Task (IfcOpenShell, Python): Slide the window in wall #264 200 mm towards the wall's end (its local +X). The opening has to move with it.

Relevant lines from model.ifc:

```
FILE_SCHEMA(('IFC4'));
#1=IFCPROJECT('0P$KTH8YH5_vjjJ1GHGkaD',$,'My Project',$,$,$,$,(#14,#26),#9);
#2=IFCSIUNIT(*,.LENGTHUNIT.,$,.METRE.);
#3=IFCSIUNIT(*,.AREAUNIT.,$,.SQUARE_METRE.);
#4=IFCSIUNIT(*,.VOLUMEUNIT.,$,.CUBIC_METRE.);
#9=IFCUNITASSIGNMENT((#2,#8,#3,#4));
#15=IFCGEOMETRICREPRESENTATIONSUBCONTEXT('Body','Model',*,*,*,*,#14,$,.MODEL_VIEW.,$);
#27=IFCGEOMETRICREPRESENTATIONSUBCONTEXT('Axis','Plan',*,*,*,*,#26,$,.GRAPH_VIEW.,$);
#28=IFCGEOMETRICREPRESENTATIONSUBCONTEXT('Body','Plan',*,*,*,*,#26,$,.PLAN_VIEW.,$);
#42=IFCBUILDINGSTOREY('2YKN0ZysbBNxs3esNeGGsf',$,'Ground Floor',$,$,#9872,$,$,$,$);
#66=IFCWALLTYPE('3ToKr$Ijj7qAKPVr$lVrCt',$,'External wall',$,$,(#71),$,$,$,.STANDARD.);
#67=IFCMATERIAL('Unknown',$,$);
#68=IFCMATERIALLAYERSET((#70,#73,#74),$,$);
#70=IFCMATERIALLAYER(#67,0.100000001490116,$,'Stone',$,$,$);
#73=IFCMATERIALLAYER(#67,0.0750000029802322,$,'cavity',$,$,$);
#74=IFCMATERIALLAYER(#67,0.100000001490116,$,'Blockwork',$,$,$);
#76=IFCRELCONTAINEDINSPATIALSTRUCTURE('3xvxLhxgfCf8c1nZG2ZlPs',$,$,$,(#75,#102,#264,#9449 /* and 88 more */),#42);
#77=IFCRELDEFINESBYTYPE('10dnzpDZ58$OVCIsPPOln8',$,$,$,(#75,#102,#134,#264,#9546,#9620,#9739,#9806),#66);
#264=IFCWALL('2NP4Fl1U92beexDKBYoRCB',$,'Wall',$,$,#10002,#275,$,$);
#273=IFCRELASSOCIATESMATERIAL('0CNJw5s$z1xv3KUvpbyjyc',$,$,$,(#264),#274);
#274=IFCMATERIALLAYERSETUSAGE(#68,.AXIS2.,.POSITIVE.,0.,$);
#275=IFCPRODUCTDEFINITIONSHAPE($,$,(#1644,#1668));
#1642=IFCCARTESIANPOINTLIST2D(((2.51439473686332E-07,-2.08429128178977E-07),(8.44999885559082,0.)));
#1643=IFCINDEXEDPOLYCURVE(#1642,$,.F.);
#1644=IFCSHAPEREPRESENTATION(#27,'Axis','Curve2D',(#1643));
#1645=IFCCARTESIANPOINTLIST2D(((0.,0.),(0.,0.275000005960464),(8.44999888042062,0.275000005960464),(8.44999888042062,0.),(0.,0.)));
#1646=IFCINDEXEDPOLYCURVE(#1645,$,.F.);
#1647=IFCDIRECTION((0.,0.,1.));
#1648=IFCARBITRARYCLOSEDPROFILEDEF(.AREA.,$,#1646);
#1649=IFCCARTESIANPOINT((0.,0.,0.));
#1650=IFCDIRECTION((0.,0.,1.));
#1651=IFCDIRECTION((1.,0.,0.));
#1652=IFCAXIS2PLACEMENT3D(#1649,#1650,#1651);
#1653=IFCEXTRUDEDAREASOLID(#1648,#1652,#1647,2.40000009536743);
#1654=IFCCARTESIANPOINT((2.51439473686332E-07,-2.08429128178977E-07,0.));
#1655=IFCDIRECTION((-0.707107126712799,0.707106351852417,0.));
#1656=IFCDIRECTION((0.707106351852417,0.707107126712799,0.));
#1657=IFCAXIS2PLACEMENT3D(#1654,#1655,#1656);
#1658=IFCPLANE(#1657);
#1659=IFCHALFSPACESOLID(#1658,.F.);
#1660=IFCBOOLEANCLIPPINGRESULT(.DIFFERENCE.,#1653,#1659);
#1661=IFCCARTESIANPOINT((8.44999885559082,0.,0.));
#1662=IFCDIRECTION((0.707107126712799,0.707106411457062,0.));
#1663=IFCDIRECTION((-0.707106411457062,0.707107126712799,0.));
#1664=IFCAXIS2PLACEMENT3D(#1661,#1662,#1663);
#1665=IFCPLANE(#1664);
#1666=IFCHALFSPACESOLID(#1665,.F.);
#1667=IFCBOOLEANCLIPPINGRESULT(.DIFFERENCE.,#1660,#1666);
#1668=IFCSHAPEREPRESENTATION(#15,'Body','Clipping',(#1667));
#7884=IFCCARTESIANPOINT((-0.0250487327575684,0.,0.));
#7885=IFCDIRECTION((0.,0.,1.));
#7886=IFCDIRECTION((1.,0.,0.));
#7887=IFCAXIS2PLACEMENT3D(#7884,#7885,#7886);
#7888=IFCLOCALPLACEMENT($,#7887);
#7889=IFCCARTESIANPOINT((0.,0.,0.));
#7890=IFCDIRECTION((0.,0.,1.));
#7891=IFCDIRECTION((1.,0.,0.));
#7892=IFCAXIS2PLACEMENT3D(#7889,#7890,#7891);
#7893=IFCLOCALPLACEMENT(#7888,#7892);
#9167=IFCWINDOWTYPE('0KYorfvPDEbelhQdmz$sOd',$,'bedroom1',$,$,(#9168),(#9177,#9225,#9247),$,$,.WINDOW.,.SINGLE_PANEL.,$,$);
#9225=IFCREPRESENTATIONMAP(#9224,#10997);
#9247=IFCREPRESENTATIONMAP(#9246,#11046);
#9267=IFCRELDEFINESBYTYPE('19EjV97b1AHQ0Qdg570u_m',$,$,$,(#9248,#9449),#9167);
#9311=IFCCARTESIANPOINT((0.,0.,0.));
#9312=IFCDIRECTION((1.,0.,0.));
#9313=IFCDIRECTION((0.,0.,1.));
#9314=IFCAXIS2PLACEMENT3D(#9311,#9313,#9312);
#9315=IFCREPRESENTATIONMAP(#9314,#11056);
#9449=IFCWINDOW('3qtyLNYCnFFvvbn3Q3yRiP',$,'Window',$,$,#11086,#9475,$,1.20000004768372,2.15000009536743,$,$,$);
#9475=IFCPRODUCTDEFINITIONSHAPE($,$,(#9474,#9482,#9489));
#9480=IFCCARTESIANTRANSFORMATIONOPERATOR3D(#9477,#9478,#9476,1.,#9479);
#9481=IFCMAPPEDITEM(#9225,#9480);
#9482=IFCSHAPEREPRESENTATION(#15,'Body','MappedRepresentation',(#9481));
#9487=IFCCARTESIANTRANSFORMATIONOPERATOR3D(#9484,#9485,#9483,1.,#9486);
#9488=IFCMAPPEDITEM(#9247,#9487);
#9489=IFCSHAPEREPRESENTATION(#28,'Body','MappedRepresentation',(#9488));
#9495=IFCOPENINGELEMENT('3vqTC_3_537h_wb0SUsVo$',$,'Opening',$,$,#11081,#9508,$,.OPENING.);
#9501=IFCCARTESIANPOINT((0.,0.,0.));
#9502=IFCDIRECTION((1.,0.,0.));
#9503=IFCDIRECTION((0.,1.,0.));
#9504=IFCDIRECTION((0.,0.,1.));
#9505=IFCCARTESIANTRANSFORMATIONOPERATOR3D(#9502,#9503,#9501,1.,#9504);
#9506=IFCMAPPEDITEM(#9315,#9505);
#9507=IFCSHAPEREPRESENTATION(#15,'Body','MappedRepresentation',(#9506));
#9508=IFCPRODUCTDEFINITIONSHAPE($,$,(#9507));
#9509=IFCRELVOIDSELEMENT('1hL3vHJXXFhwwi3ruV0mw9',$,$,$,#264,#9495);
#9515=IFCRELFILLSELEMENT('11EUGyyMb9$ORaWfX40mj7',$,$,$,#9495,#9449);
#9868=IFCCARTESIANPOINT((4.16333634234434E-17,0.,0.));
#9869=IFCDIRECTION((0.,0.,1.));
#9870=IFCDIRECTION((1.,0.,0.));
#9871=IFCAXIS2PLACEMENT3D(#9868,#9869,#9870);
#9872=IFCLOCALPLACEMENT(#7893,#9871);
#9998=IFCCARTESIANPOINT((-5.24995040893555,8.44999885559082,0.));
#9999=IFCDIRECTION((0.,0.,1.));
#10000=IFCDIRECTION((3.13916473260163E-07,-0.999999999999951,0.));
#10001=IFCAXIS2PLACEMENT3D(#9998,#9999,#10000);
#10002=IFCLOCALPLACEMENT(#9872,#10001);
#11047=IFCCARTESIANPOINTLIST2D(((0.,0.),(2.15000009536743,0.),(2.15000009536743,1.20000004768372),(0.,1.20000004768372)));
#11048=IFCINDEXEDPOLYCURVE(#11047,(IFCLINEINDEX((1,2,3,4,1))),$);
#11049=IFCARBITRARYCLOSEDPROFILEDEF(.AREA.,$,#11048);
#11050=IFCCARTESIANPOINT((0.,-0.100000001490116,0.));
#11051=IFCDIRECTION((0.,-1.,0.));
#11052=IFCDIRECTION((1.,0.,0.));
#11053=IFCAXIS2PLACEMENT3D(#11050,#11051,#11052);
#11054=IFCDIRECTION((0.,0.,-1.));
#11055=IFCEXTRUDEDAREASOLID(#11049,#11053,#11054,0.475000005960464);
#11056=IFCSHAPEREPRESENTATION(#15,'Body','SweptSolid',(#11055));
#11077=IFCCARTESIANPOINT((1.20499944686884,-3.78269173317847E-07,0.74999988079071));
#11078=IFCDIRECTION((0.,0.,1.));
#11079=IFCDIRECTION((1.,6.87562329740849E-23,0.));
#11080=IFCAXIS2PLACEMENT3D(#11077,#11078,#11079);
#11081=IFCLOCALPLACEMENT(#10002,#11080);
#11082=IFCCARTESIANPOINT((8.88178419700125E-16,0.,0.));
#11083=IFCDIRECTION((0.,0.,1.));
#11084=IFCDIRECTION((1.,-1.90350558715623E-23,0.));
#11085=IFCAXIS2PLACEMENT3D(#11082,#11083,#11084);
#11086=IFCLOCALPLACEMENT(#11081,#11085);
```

```python
import ifcopenshell
import ifcopenshell.api.geometry
import ifcopenshell.util.placement
import ifcopenshell.util.unit

model = ifcopenshell.open("model.ifc")
unit_scale = ifcopenshell.util.unit.calculate_unit_scale(model)

window = model.by_id(9449)
opening = window.FillsVoids[0].RelatingOpeningElement
wall = opening.VoidsElements[0].RelatingBuildingElement

wall_matrix = ifcopenshell.util.placement.get_local_placement(wall.ObjectPlacement)
shift = wall_matrix[:3, 0] * 0.2 / unit_scale
before = ifcopenshell.util.placement.get_local_placement(window.ObjectPlacement)[:3, 3].copy()

# The window is placed relative to its opening, so it follows when the opening moves.
matrix = ifcopenshell.util.placement.get_local_placement(opening.ObjectPlacement)
matrix[:3, 3] += shift
ifcopenshell.api.geometry.edit_object_placement(
    model, product=opening, matrix=matrix, is_si=False, should_transform_children=True
)

after = ifcopenshell.util.placement.get_local_placement(window.ObjectPlacement)[:3, 3]
print("window moved by", (after - before).round(3) + 0.0)

model.write("model_v2.ifc")
```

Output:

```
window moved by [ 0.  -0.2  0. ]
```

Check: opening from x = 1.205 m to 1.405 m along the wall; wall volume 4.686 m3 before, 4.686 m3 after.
